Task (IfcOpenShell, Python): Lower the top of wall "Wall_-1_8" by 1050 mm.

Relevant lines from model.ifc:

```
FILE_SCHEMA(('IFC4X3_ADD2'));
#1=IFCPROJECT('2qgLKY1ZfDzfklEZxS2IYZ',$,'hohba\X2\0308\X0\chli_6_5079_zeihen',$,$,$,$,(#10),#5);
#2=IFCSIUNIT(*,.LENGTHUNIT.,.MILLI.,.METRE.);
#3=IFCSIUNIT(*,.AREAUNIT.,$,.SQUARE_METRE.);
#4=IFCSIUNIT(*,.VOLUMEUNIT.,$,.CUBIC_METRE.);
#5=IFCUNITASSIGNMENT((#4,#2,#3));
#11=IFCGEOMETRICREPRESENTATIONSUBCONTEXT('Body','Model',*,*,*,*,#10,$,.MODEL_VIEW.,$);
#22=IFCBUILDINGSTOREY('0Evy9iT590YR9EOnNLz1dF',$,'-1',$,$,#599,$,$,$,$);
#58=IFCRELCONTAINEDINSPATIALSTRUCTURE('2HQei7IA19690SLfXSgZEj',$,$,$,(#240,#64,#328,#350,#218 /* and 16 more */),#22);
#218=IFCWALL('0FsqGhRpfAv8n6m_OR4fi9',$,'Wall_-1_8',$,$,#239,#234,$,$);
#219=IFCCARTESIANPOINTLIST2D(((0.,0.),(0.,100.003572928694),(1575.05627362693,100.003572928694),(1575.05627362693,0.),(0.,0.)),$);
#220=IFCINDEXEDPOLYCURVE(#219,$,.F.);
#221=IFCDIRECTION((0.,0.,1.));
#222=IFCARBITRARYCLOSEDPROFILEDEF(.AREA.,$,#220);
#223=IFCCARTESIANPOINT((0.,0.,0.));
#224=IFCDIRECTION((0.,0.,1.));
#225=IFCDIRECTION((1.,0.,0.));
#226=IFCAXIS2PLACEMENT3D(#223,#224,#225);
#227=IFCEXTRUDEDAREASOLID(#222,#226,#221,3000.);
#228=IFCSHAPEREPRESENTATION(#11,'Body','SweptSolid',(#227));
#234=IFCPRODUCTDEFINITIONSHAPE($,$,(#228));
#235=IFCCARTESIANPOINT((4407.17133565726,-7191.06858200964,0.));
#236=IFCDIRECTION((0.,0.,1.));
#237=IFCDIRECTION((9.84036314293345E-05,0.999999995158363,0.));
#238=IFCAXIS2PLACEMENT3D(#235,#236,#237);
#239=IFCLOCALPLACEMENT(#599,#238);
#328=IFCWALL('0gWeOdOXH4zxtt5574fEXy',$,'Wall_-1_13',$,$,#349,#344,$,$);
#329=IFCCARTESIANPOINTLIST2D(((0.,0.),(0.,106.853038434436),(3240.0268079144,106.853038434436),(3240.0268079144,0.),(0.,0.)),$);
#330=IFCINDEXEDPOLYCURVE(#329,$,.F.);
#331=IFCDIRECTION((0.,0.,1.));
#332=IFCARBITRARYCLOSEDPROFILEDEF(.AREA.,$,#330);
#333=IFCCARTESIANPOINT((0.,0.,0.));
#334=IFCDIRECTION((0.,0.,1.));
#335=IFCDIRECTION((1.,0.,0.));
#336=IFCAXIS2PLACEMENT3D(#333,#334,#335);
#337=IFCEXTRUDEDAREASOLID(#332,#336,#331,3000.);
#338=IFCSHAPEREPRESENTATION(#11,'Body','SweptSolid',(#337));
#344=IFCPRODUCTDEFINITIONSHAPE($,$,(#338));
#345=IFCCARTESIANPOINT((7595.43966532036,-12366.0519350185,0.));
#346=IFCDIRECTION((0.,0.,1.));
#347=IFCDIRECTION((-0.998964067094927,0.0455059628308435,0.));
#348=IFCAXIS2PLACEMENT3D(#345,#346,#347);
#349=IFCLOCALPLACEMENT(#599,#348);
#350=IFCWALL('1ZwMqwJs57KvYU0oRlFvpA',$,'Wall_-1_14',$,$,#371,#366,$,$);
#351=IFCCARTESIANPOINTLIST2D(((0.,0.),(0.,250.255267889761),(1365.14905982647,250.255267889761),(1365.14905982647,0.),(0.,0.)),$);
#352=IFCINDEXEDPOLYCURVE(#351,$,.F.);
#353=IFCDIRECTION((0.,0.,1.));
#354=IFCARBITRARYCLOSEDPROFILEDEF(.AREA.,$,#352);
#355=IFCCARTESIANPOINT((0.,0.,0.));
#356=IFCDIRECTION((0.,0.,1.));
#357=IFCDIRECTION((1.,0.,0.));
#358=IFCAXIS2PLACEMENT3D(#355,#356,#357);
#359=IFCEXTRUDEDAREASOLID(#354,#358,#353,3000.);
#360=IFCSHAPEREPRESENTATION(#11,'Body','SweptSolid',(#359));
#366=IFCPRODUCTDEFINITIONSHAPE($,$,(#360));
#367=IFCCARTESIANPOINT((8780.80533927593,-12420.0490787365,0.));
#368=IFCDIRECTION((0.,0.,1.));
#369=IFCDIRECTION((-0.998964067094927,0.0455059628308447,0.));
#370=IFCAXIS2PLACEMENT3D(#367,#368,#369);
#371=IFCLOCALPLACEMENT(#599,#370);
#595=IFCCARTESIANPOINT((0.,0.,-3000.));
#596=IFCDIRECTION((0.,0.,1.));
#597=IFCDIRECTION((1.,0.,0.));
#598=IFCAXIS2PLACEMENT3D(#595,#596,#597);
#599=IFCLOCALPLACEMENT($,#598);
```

```python
import ifcopenshell
import ifcopenshell.geom
import ifcopenshell.util.representation
import ifcopenshell.util.shape

model = ifcopenshell.open("model.ifc")
settings = ifcopenshell.geom.settings()


def volume(element):
    """Net volume in cubic metres, openings subtracted."""
    shape = ifcopenshell.geom.create_shape(settings, element)
    return ifcopenshell.util.shape.get_volume(shape.geometry)


wall = model.by_guid("0FsqGhRpfAv8n6m_OR4fi9")
before = volume(wall)

body = ifcopenshell.util.representation.get_representation(wall, "Model", "Body")
solid = body.Items[0]
old_height = solid.Depth
solid.Depth -= 1050.0
after = volume(wall)

print(f"height {old_height:g} -> {solid.Depth:g}, volume {before:.3f} -> {after:.3f} m3")

model.write("model_edited.ifc")
```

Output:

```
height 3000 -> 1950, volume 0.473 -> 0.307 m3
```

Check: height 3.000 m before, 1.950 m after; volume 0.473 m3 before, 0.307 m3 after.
